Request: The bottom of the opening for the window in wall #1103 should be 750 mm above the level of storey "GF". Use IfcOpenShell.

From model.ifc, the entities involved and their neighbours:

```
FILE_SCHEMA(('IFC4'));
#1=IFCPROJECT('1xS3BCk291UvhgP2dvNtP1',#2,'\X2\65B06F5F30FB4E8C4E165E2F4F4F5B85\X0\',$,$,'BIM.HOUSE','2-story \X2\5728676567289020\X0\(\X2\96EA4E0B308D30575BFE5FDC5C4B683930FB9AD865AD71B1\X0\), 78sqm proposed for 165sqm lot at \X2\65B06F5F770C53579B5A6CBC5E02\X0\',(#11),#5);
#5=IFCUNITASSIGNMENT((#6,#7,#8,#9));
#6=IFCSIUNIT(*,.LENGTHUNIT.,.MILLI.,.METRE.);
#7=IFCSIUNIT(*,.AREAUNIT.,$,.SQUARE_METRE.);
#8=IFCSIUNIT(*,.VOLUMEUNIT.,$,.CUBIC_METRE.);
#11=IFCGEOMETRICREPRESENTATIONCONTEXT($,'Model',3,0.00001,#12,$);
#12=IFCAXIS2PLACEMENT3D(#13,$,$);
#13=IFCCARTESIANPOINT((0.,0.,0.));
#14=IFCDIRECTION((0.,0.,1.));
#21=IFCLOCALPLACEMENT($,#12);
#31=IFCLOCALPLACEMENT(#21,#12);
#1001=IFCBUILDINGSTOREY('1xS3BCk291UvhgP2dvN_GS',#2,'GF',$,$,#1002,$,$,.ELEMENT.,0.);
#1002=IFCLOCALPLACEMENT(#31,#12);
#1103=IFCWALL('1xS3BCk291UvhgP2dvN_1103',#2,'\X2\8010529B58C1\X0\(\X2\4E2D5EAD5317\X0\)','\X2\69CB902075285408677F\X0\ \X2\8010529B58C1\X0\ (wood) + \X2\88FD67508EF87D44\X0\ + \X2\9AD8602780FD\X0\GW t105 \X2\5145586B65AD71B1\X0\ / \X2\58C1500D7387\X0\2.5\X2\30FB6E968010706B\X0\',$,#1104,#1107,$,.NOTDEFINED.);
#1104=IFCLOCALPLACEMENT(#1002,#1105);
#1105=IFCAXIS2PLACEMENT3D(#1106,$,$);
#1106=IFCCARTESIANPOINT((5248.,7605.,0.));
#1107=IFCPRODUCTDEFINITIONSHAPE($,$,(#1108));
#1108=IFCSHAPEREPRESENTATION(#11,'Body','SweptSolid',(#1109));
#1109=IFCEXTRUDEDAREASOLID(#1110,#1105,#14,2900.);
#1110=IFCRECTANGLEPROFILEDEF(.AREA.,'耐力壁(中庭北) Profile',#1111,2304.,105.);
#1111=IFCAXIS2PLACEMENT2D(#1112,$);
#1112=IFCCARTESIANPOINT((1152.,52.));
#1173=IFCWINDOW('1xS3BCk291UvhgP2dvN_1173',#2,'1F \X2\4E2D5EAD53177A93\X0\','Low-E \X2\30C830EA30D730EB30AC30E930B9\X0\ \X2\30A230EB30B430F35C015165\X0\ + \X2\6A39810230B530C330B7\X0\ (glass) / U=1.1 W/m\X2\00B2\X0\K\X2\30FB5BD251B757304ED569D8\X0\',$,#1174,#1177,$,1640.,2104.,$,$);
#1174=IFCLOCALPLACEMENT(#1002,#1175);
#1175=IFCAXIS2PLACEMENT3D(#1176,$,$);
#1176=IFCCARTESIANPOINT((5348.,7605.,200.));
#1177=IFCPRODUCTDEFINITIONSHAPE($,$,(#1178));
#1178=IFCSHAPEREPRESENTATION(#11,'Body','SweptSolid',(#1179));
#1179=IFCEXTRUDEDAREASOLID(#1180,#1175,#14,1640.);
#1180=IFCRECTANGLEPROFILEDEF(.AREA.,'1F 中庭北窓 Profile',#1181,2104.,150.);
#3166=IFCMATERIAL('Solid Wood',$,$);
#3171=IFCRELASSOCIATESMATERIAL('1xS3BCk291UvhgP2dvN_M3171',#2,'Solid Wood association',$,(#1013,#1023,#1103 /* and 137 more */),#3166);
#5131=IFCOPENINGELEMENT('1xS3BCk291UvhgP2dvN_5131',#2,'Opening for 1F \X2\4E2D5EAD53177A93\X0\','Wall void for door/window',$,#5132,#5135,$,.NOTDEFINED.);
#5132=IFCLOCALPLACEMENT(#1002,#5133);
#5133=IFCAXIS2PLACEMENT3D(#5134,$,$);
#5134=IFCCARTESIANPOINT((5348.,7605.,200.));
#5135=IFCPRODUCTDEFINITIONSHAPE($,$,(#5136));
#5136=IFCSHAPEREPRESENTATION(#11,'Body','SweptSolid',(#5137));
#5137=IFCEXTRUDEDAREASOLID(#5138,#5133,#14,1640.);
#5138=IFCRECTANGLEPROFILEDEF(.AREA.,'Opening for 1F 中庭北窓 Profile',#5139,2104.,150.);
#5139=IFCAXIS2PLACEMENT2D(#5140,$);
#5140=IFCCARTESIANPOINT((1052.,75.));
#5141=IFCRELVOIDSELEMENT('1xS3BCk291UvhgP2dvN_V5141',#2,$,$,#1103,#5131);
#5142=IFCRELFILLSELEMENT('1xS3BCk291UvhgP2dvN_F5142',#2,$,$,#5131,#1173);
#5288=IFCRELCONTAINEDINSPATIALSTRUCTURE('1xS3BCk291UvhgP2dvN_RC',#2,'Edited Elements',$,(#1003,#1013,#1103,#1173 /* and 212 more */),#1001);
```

```python
import numpy as np
import ifcopenshell
import ifcopenshell.api.geometry
import ifcopenshell.geom
import ifcopenshell.util.element
import ifcopenshell.util.placement
import ifcopenshell.util.shape
import ifcopenshell.util.unit

model = ifcopenshell.open("model.ifc")
unit_scale = ifcopenshell.util.unit.calculate_unit_scale(model)

window = model.by_guid("1xS3BCk291UvhgP2dvN_1173")
opening = window.FillsVoids[0].RelatingOpeningElement
storey = ifcopenshell.util.element.get_container(window, ifc_class="IfcBuildingStorey")
level = ifcopenshell.util.placement.get_local_placement(storey.ObjectPlacement)[2, 3]

# The opening's origin need not be at the sill, so measure its lowest point.
shape = ifcopenshell.geom.create_shape(ifcopenshell.geom.settings(), opening)
bottom = ifcopenshell.util.shape.get_shape_bottom_elevation(shape, shape.geometry) / unit_scale
dz = level + 0.75 / unit_scale - bottom

shift = np.array([0.0, 0.0, dz])
# The window is not placed relative to its opening, so move both.
for product in (opening, window):
    matrix = ifcopenshell.util.placement.get_local_placement(product.ObjectPlacement)
    matrix[:3, 3] += shift
    ifcopenshell.api.geometry.edit_object_placement(model, product=product, matrix=matrix, is_si=False)

print(f"moved by {dz * unit_scale:+.3f} m")

model.write("model_edited.ifc")
```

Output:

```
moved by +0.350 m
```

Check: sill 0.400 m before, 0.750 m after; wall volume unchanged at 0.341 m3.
